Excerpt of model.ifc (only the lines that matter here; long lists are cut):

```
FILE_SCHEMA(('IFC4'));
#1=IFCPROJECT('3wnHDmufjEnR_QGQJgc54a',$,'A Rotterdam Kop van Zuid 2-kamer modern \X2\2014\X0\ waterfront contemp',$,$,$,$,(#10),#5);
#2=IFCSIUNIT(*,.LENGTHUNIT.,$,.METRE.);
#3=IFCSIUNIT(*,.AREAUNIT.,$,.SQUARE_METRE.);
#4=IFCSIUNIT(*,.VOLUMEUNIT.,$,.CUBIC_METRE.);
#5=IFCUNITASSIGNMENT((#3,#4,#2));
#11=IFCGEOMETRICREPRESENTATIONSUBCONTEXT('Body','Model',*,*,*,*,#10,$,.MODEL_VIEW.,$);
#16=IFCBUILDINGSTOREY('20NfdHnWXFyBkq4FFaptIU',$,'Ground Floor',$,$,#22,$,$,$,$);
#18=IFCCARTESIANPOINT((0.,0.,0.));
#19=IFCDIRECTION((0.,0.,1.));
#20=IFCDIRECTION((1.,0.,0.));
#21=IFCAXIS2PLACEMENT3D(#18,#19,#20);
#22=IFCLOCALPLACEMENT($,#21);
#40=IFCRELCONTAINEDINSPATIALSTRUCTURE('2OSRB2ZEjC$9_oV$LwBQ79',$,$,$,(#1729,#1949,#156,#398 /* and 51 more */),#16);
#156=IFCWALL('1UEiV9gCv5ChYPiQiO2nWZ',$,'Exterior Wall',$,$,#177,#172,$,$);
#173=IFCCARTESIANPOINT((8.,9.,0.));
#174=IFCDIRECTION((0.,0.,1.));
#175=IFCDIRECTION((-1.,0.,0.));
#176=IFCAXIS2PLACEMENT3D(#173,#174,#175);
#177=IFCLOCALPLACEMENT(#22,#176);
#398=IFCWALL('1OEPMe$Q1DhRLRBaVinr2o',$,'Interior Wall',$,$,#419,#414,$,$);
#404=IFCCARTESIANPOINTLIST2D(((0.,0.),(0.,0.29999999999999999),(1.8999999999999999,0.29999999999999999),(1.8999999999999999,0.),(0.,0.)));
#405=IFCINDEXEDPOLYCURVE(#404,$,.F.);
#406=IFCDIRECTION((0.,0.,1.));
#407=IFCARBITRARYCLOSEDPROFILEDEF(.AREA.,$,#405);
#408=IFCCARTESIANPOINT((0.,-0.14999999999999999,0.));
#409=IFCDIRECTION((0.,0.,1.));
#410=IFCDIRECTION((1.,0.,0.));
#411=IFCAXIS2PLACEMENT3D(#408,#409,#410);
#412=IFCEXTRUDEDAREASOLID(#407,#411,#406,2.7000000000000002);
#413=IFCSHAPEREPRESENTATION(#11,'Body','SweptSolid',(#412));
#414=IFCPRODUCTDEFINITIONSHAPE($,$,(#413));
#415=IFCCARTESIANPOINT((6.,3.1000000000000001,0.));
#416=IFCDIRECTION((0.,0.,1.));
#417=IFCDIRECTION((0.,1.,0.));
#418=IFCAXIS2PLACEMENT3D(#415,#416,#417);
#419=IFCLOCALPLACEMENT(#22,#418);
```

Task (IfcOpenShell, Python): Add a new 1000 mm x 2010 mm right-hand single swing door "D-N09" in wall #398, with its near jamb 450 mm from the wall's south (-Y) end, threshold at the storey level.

```python
import numpy as np
import ifcopenshell
import ifcopenshell.api.feature
import ifcopenshell.api.geometry
import ifcopenshell.api.root
import ifcopenshell.api.spatial
import ifcopenshell.geom
import ifcopenshell.util.element
import ifcopenshell.util.placement
import ifcopenshell.util.representation
import ifcopenshell.util.shape
import ifcopenshell.util.unit

model = ifcopenshell.open("model.ifc")
unit_scale = ifcopenshell.util.unit.calculate_unit_scale(model)
settings = ifcopenshell.geom.settings()


def volume(element):
    """Net volume in cubic metres, openings subtracted."""
    shape = ifcopenshell.geom.create_shape(settings, element)
    return ifcopenshell.util.shape.get_volume(shape.geometry)


wall = model.by_guid("1OEPMe$Q1DhRLRBaVinr2o")
storey = ifcopenshell.util.element.get_container(wall, ifc_class="IfcBuildingStorey")
context = ifcopenshell.util.representation.get_context(model, "Model", "Body", "MODEL_VIEW")
before = volume(wall)

width, height, from_end, sill = 1, 2.01, 0.45, 0.0  # metres

# The wall runs along its own X axis, and the end named is its -X end.
wall_shape = ifcopenshell.geom.create_shape(settings, wall)
x, y, z = ifcopenshell.util.shape.get_vertices(wall_shape.geometry).T
start = x.min() + from_end
face, thickness = float(y.min()), float(y.max() - y.min())
wall_matrix = ifcopenshell.util.placement.get_local_placement(wall.ObjectPlacement)
level = ifcopenshell.util.placement.get_local_placement(storey.ObjectPlacement)[2, 3]


def in_wall(x, y):
    """Placement at x, y metres in the wall's axes, at sill height."""
    matrix = wall_matrix.copy()
    matrix[:, 3] = wall_matrix @ np.array([x / unit_scale, y / unit_scale, 0.0, 1.0])
    matrix[2, 3] = level + sill / unit_scale
    return matrix


# Opening: a box that overshoots both wall faces by 50 mm.
opening = ifcopenshell.api.root.create_entity(model, ifc_class="IfcOpeningElement", predefined_type="OPENING")
box = ifcopenshell.api.geometry.add_wall_representation(
    model, context=context, length=width, height=height, thickness=thickness + 0.1
)
ifcopenshell.api.geometry.assign_representation(model, product=opening, representation=box)
ifcopenshell.api.geometry.edit_object_placement(model, product=opening, matrix=in_wall(start, face - 0.05), is_si=False)
ifcopenshell.api.feature.add_feature(model, feature=opening, element=wall)

door = ifcopenshell.api.root.create_entity(model, ifc_class="IfcDoor", name="D-N09", predefined_type="DOOR")
door.OverallWidth, door.OverallHeight = width / unit_scale, height / unit_scale
door.OperationType = "SINGLE_SWING_RIGHT"
body = ifcopenshell.api.geometry.add_door_representation(
    model,
    context=context,
    overall_width=door.OverallWidth,
    overall_height=door.OverallHeight,
    operation_type="SINGLE_SWING_RIGHT",
    lining_properties={"LiningDepth": thickness / unit_scale, "ThresholdDepth": thickness / unit_scale},
)
ifcopenshell.api.geometry.assign_representation(model, product=door, representation=body)
ifcopenshell.api.spatial.assign_container(model, products=[door], relating_structure=storey)
ifcopenshell.api.feature.add_filling(model, opening=opening, element=door)

# The lining spans the wall, so the door starts at the wall face.
ifcopenshell.api.geometry.edit_object_placement(model, product=door, matrix=in_wall(start, face), is_si=False)

after = volume(wall)

print(f"wall volume {before:.3f} -> {after:.3f} m3")

model.write("model-out.ifc")
```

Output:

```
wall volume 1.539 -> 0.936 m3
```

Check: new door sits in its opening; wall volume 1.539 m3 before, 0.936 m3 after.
